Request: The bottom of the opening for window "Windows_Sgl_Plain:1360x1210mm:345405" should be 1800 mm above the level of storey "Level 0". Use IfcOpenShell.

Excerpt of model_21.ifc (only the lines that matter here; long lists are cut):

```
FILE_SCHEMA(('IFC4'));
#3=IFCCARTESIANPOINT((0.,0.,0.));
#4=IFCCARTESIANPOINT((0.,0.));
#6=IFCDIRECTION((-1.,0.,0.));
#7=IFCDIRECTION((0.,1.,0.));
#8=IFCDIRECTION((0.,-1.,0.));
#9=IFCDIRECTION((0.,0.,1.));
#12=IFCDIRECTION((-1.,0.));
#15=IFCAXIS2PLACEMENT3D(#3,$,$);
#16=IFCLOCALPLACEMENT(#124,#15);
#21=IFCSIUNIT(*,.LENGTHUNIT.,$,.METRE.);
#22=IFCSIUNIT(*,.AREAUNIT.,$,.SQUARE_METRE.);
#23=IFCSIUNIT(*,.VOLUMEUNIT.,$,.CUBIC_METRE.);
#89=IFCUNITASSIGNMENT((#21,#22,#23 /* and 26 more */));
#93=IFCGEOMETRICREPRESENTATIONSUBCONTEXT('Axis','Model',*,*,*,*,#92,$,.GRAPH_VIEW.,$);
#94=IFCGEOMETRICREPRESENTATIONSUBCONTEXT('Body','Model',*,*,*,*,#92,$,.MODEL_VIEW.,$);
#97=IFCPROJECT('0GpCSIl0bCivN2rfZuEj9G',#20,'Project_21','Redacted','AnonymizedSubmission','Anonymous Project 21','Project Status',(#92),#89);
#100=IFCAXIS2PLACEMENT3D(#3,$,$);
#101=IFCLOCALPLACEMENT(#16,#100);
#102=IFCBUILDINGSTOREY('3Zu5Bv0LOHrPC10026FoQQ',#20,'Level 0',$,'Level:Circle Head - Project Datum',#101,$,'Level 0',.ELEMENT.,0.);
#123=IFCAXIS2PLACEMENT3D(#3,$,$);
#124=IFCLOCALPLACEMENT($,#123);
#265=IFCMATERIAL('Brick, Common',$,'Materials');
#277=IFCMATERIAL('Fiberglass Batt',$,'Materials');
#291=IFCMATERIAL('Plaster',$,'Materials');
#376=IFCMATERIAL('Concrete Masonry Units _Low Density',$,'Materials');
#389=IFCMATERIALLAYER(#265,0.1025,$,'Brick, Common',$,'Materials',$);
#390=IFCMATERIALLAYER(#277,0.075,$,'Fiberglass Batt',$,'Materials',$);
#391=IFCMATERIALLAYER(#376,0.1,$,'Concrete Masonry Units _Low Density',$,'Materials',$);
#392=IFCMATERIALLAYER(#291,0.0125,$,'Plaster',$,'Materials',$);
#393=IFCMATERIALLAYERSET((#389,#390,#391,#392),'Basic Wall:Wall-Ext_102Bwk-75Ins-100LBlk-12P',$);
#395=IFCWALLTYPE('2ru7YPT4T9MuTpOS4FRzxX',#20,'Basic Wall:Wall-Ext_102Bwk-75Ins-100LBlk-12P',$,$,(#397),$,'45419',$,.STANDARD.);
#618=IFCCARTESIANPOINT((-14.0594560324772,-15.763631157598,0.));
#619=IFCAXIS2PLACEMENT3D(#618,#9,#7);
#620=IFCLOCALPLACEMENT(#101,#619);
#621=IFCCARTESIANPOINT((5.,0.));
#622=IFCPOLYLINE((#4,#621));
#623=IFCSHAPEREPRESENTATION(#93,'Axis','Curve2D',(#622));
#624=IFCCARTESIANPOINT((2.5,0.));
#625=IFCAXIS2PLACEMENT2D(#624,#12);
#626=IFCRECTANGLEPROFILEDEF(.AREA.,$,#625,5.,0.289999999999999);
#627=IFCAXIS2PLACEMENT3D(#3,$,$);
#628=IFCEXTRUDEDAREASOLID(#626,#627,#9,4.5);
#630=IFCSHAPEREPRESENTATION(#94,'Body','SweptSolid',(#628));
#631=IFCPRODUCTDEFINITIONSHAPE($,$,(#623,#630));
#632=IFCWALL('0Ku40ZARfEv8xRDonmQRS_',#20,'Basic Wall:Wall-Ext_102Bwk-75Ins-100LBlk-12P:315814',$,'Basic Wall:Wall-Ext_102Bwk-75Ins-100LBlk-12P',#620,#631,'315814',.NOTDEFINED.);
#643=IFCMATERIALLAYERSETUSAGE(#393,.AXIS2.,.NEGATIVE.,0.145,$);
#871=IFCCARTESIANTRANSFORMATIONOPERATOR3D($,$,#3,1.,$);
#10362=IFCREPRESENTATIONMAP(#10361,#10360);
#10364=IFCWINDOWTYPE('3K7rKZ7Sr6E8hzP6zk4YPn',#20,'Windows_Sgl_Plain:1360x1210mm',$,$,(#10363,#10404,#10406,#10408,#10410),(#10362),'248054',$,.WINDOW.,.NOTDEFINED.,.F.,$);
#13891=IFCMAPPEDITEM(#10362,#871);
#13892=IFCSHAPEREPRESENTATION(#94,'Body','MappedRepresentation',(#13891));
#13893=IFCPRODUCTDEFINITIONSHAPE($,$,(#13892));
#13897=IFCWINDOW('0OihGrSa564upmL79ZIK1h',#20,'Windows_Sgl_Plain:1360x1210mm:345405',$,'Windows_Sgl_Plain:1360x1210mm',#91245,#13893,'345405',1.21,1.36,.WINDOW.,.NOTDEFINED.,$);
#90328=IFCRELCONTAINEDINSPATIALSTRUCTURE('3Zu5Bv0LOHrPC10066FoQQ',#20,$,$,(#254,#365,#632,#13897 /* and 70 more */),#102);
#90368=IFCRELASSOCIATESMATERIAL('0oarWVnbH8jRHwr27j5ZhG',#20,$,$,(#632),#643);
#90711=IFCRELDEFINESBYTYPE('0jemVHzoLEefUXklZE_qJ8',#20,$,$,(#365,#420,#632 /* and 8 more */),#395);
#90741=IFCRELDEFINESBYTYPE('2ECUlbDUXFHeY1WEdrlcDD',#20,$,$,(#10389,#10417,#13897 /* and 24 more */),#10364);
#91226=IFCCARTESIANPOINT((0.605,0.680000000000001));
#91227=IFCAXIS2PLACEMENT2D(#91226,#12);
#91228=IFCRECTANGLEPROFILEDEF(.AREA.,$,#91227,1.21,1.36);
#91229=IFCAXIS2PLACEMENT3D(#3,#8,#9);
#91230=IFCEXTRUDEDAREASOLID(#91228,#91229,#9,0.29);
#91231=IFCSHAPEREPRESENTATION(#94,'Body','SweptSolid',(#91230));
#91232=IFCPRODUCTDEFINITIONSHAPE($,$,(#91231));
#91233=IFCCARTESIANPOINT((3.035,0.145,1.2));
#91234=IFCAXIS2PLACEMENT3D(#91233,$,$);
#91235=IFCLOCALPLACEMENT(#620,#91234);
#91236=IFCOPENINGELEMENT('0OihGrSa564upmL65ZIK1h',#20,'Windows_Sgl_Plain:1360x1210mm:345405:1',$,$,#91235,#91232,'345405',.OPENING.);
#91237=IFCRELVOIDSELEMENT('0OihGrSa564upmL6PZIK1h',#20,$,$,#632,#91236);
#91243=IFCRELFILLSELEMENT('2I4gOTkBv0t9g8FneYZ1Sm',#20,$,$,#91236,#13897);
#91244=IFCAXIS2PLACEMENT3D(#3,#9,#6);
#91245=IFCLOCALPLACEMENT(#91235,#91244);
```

```python
import numpy as np
import ifcopenshell
import ifcopenshell.api.geometry
import ifcopenshell.geom
import ifcopenshell.util.element
import ifcopenshell.util.placement
import ifcopenshell.util.shape
import ifcopenshell.util.unit

model = ifcopenshell.open("model_21.ifc")
unit_scale = ifcopenshell.util.unit.calculate_unit_scale(model)

window = model.by_guid("0OihGrSa564upmL79ZIK1h")
opening = window.FillsVoids[0].RelatingOpeningElement
storey = ifcopenshell.util.element.get_container(window, ifc_class="IfcBuildingStorey")
level = ifcopenshell.util.placement.get_local_placement(storey.ObjectPlacement)[2, 3]

# The opening's origin need not be at the sill, so measure its lowest point.
shape = ifcopenshell.geom.create_shape(ifcopenshell.geom.settings(), opening)
bottom = ifcopenshell.util.shape.get_shape_bottom_elevation(shape, shape.geometry) / unit_scale
dz = level + 1.8 / unit_scale - bottom

shift = np.array([0.0, 0.0, dz])
# The window is placed relative to its opening, so it follows when the opening moves.
matrix = ifcopenshell.util.placement.get_local_placement(opening.ObjectPlacement)
matrix[:3, 3] += shift
ifcopenshell.api.geometry.edit_object_placement(
    model, product=opening, matrix=matrix, is_si=False, should_transform_children=True
)

print(f"moved by {dz * unit_scale:+.3f} m")

model.write("model_21-out.ifc")
```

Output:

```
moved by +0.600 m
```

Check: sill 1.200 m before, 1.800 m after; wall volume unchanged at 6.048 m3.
